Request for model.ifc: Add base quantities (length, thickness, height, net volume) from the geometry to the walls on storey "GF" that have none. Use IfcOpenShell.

First a look at what the model holds.

```python
import ifcopenshell
import ifcopenshell.util.element
import ifcopenshell.util.unit

model = ifcopenshell.open("model.ifc")
print(model.schema)
for unit_type in ("LENGTHUNIT", "AREAUNIT", "VOLUMEUNIT"):
    print(unit_type, ifcopenshell.util.unit.calculate_unit_scale(model, unit_type))
storey = next(s for s in model.by_type("IfcBuildingStorey") if s.Name == "GF")
walls = [e for e in ifcopenshell.util.element.get_decomposition(storey) if e.is_a("IfcWall")]
for e in sorted(walls, key=lambda e: e.id()):
    print(e.id(), e.is_a(), e.Name, list(ifcopenshell.util.element.get_psets(e, qtos_only=True)), sep=" | ")
```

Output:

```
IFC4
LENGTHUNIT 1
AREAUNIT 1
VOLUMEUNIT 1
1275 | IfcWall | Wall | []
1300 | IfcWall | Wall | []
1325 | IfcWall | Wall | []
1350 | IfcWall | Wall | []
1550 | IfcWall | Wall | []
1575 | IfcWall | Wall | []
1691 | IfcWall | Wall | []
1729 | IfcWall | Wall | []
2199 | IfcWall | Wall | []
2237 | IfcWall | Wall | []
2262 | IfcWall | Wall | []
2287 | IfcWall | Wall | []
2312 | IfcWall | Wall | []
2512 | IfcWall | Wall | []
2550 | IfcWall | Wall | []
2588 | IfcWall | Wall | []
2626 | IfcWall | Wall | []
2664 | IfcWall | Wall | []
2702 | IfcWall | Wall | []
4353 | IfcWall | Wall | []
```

```python
import ifcopenshell
import ifcopenshell.api.pset
import ifcopenshell.geom
import ifcopenshell.util.element
import ifcopenshell.util.shape
import ifcopenshell.util.unit

model = ifcopenshell.open("model.ifc")
unit_scale = ifcopenshell.util.unit.calculate_unit_scale(model)
volume_scale = ifcopenshell.util.unit.calculate_unit_scale(model, "VOLUMEUNIT")
settings = ifcopenshell.geom.settings()

storey = next(s for s in model.by_type("IfcBuildingStorey") if s.Name == "GF")
walls = [e for e in ifcopenshell.util.element.get_decomposition(storey) if e.is_a("IfcWall")]

for e in sorted(walls, key=lambda e: e.id()):
    if ifcopenshell.util.element.get_psets(e, qtos_only=True, should_inherit=False):
        continue
    # Geometry comes back in metres, in the element's own axes.
    shape = ifcopenshell.geom.create_shape(settings, e)
    values = {
        "Length": ifcopenshell.util.shape.get_x(shape.geometry) / unit_scale,
        "Width": ifcopenshell.util.shape.get_y(shape.geometry) / unit_scale,
        "Height": ifcopenshell.util.shape.get_z(shape.geometry) / unit_scale,
        "NetVolume": ifcopenshell.util.shape.get_volume(shape.geometry) / volume_scale,
    }
    qto = ifcopenshell.api.pset.add_qto(model, product=e, name="Qto_WallBaseQuantities")
    ifcopenshell.api.pset.edit_qto(model, qto=qto, properties=values)
    print(e.id(), {k: round(v, 3) for k, v in values.items()})

model.write("model_v2.ifc")
```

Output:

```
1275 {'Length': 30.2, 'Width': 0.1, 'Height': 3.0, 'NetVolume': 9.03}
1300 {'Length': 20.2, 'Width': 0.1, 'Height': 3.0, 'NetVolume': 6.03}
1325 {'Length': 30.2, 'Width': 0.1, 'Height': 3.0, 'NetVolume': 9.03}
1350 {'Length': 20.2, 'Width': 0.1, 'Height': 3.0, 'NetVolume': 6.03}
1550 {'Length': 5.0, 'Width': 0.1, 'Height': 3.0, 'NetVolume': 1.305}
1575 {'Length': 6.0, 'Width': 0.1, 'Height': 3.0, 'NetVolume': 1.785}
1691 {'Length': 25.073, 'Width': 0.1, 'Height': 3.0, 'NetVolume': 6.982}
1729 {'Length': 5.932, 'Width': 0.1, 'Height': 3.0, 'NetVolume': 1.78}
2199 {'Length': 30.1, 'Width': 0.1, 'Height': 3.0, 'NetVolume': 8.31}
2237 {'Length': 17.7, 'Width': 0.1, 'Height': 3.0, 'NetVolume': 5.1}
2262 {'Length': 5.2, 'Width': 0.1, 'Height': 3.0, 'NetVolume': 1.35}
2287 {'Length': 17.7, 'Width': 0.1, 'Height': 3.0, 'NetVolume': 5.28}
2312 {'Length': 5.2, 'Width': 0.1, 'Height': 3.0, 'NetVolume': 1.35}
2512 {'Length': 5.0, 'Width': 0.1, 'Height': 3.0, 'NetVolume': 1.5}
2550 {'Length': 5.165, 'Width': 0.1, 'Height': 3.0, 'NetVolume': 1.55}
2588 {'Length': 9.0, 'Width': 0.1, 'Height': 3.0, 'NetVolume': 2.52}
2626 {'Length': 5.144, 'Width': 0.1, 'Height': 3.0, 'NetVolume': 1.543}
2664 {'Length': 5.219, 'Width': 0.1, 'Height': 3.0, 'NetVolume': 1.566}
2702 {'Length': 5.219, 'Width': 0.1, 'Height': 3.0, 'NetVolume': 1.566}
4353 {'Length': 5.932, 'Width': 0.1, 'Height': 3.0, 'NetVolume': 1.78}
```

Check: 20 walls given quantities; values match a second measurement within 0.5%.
